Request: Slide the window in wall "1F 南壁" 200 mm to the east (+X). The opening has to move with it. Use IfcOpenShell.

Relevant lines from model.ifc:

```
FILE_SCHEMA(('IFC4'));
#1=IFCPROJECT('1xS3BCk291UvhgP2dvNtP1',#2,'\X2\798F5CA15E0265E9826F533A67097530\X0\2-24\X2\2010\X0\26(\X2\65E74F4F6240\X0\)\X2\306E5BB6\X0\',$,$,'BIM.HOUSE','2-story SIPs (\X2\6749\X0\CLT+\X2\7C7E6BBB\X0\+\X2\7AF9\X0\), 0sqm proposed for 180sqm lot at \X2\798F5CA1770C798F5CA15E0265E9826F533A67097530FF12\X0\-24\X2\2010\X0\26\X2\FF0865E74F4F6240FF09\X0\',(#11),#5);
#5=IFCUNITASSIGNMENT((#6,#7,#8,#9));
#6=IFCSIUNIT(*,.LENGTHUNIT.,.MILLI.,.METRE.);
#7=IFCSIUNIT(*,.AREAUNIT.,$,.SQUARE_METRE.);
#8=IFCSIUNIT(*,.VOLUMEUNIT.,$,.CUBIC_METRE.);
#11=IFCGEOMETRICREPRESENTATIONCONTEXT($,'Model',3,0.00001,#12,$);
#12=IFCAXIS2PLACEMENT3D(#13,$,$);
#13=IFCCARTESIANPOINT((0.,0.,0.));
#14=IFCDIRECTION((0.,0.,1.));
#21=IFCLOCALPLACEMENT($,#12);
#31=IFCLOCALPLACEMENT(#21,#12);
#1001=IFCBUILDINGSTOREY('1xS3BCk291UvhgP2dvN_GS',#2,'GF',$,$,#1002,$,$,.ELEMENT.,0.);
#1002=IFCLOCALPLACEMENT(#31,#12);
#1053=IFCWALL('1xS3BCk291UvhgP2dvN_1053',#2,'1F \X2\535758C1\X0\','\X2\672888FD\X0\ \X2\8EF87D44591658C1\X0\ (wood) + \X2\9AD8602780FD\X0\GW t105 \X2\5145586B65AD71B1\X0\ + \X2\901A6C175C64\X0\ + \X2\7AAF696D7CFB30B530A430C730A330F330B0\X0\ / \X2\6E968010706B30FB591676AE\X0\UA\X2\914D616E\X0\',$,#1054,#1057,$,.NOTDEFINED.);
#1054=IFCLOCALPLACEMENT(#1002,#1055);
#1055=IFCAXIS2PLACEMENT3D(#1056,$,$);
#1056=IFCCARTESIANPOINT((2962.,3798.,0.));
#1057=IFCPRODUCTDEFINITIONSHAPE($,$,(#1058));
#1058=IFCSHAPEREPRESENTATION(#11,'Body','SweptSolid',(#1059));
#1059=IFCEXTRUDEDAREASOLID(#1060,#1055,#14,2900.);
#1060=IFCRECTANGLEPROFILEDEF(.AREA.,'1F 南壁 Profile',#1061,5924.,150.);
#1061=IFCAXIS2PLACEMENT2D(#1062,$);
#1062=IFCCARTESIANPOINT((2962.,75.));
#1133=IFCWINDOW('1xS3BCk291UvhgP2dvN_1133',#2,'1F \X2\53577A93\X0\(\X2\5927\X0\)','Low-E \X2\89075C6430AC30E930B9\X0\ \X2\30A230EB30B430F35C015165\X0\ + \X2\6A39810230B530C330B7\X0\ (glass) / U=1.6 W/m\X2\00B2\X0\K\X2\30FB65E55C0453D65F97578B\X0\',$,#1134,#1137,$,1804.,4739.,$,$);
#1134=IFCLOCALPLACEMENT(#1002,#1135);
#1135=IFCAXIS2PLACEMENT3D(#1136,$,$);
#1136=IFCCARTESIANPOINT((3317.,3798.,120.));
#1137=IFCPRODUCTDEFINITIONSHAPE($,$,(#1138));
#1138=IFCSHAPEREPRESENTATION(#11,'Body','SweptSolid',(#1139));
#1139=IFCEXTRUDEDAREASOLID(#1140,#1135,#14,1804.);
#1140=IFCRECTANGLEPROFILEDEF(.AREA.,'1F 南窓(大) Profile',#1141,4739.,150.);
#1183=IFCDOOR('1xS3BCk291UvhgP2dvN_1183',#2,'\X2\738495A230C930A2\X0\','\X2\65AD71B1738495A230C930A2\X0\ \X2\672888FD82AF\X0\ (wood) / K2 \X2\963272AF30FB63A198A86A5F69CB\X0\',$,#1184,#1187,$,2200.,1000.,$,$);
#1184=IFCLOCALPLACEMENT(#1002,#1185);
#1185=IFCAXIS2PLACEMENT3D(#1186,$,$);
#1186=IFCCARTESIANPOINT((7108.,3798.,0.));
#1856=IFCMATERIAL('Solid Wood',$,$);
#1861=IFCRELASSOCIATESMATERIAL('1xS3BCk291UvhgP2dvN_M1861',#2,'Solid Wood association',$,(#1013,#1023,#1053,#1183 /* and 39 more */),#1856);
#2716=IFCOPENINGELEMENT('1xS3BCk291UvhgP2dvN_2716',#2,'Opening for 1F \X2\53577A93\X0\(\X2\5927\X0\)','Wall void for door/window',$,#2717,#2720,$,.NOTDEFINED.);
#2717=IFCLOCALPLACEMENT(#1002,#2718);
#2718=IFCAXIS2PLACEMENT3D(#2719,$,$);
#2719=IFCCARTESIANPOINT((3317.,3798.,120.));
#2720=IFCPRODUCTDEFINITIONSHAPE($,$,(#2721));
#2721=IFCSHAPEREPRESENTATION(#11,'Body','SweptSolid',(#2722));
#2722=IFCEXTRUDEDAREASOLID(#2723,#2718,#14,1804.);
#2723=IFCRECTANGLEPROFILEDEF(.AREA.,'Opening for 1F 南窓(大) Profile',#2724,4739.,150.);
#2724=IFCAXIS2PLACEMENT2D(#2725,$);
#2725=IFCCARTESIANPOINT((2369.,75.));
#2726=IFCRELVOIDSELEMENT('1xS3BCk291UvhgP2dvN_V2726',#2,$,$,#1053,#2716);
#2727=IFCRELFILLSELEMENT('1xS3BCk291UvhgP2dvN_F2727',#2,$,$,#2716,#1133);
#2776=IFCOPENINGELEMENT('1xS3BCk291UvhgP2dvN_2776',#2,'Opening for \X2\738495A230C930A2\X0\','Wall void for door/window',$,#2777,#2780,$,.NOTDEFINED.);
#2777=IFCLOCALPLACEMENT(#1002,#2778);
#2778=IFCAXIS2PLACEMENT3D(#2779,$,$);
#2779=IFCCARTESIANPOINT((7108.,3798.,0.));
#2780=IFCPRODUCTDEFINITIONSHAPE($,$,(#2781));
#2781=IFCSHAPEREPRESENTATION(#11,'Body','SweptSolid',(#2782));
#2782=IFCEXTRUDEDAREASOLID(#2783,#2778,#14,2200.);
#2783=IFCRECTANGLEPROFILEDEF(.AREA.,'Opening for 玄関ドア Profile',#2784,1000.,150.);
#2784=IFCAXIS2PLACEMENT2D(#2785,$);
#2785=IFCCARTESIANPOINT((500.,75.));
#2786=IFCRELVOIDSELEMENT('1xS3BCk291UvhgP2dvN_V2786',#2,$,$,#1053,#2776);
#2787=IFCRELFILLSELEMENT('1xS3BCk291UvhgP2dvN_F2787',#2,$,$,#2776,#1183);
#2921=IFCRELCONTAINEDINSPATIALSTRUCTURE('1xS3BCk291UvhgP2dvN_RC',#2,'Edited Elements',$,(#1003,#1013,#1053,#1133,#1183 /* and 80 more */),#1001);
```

```python
import ifcopenshell
import ifcopenshell.api.geometry
import ifcopenshell.util.placement

model = ifcopenshell.open("model.ifc")

window = model.by_guid("1xS3BCk291UvhgP2dvN_1133")
opening = window.FillsVoids[0].RelatingOpeningElement
wall = opening.VoidsElements[0].RelatingBuildingElement

wall_matrix = ifcopenshell.util.placement.get_local_placement(wall.ObjectPlacement)
shift = wall_matrix[:3, 0] * 200.0
before = ifcopenshell.util.placement.get_local_placement(window.ObjectPlacement)[:3, 3].copy()

# The window is not placed relative to its opening, so move both.
for product in (opening, window):
    matrix = ifcopenshell.util.placement.get_local_placement(product.ObjectPlacement)
    matrix[:3, 3] += shift
    ifcopenshell.api.geometry.edit_object_placement(model, product=product, matrix=matrix, is_si=False)

after = ifcopenshell.util.placement.get_local_placement(window.ObjectPlacement)[:3, 3]
print("window moved by", (after - before).round(3) + 0.0)

model.write("model-out.ifc")
```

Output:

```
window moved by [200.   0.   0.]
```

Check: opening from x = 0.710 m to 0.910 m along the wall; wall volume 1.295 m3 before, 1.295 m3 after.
